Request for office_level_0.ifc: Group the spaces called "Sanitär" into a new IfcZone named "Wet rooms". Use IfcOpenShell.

First a look at what the model holds.

```python
import ifcopenshell

model = ifcopenshell.open("office_level_0.ifc")
print(model.schema)
seen = {}
for space in model.by_type("IfcSpace"):
    seen[space.LongName] = seen.get(space.LongName, 0) + 1
for name, count in sorted(seen.items(), key=str):
    print(count, "x", name)
print("zones:", [z.Name for z in model.by_type("IfcZone")][:20])
```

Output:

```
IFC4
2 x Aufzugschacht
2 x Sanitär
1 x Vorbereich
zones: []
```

```python
import ifcopenshell
import ifcopenshell.api.group
import ifcopenshell.api.root

model = ifcopenshell.open("office_level_0.ifc")

names = {"Sanitär"}
spaces = [s for s in model.by_type("IfcSpace") if s.LongName in names]

zone = ifcopenshell.api.root.create_entity(model, ifc_class="IfcZone", name="Wet rooms")
ifcopenshell.api.group.assign_group(model, products=spaces, group=zone)
print(len(spaces), "spaces in", zone.Name)

model.write("office_level_0_updated.ifc")
```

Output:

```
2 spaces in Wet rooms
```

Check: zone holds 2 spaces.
